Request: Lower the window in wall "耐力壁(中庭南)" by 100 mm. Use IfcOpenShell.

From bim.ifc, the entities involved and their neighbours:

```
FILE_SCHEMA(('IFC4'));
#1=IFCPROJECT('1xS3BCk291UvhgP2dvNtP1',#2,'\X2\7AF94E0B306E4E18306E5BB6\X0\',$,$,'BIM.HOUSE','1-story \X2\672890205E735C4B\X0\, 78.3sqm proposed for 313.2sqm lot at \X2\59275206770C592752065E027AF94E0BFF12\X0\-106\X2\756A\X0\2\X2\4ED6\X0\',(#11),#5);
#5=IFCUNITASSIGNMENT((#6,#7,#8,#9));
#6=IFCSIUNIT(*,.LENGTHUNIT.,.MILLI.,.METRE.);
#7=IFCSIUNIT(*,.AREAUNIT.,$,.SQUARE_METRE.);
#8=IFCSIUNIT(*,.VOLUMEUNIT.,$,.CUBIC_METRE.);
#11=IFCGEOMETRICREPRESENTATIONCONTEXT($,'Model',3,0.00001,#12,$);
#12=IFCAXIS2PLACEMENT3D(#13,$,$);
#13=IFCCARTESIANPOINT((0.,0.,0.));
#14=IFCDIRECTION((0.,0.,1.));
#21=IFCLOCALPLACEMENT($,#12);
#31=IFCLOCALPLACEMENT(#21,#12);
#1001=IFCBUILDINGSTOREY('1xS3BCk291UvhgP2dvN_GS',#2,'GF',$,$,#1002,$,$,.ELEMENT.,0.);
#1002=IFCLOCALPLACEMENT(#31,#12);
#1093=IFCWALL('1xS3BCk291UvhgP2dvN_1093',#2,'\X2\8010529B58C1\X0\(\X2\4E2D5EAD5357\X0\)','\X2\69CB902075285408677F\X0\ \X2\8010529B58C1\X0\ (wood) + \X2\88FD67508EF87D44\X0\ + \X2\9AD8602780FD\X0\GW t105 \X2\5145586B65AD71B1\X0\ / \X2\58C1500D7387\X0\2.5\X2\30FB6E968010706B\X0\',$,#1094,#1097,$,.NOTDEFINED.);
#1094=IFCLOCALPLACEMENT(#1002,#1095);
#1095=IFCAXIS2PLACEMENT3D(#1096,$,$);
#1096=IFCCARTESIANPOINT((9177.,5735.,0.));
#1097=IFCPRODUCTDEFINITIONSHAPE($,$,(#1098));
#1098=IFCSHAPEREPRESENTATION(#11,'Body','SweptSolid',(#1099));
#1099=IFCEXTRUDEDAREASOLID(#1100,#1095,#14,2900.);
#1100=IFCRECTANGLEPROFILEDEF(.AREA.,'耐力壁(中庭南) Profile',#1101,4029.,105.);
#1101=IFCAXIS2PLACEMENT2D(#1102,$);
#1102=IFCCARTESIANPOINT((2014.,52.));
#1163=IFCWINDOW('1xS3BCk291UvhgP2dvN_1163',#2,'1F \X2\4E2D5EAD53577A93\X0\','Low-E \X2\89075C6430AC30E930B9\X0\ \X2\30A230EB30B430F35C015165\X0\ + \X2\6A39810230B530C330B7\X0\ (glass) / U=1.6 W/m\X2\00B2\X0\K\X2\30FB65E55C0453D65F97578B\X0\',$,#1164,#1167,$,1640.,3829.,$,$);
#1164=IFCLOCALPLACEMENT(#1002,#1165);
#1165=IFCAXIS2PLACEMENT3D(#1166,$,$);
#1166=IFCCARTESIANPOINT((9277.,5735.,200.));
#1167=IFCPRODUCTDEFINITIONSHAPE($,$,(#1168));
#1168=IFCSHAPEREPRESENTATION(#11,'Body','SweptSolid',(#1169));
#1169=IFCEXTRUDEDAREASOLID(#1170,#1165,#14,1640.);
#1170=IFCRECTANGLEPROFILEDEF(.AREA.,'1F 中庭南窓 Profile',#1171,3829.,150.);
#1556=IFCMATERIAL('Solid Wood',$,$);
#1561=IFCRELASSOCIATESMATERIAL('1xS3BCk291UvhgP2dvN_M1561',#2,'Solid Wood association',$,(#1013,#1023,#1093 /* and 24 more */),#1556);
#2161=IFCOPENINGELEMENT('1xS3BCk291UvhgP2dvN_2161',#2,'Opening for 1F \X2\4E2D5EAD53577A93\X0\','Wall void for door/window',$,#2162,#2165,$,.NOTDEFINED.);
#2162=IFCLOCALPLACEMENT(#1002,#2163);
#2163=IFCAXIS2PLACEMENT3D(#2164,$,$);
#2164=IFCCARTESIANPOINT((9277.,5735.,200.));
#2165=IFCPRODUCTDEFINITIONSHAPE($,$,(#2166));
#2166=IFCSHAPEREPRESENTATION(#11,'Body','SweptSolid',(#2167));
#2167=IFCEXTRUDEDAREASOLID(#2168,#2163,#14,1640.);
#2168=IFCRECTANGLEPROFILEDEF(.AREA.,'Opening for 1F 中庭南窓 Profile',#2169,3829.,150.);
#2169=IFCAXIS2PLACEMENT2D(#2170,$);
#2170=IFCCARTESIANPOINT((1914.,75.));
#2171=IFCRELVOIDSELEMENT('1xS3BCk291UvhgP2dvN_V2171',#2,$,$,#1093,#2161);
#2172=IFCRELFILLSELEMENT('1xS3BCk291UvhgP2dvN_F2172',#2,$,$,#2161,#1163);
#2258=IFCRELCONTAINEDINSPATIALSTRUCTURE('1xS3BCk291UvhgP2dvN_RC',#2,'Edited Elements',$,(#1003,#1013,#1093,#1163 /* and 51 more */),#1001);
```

```python
import numpy as np
import ifcopenshell
import ifcopenshell.api.geometry
import ifcopenshell.util.placement
import ifcopenshell.util.unit

model = ifcopenshell.open("bim.ifc")
unit_scale = ifcopenshell.util.unit.calculate_unit_scale(model)

window = model.by_guid("1xS3BCk291UvhgP2dvN_1163")
opening = window.FillsVoids[0].RelatingOpeningElement
dz = -0.1 / unit_scale

shift = np.array([0.0, 0.0, dz])
# The window is not placed relative to its opening, so move both.
for product in (opening, window):
    matrix = ifcopenshell.util.placement.get_local_placement(product.ObjectPlacement)
    matrix[:3, 3] += shift
    ifcopenshell.api.geometry.edit_object_placement(model, product=product, matrix=matrix, is_si=False)

print(f"moved by {dz * unit_scale:+.3f} m")

model.write("bim_v2.ifc")
```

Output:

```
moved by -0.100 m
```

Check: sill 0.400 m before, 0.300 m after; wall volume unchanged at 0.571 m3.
